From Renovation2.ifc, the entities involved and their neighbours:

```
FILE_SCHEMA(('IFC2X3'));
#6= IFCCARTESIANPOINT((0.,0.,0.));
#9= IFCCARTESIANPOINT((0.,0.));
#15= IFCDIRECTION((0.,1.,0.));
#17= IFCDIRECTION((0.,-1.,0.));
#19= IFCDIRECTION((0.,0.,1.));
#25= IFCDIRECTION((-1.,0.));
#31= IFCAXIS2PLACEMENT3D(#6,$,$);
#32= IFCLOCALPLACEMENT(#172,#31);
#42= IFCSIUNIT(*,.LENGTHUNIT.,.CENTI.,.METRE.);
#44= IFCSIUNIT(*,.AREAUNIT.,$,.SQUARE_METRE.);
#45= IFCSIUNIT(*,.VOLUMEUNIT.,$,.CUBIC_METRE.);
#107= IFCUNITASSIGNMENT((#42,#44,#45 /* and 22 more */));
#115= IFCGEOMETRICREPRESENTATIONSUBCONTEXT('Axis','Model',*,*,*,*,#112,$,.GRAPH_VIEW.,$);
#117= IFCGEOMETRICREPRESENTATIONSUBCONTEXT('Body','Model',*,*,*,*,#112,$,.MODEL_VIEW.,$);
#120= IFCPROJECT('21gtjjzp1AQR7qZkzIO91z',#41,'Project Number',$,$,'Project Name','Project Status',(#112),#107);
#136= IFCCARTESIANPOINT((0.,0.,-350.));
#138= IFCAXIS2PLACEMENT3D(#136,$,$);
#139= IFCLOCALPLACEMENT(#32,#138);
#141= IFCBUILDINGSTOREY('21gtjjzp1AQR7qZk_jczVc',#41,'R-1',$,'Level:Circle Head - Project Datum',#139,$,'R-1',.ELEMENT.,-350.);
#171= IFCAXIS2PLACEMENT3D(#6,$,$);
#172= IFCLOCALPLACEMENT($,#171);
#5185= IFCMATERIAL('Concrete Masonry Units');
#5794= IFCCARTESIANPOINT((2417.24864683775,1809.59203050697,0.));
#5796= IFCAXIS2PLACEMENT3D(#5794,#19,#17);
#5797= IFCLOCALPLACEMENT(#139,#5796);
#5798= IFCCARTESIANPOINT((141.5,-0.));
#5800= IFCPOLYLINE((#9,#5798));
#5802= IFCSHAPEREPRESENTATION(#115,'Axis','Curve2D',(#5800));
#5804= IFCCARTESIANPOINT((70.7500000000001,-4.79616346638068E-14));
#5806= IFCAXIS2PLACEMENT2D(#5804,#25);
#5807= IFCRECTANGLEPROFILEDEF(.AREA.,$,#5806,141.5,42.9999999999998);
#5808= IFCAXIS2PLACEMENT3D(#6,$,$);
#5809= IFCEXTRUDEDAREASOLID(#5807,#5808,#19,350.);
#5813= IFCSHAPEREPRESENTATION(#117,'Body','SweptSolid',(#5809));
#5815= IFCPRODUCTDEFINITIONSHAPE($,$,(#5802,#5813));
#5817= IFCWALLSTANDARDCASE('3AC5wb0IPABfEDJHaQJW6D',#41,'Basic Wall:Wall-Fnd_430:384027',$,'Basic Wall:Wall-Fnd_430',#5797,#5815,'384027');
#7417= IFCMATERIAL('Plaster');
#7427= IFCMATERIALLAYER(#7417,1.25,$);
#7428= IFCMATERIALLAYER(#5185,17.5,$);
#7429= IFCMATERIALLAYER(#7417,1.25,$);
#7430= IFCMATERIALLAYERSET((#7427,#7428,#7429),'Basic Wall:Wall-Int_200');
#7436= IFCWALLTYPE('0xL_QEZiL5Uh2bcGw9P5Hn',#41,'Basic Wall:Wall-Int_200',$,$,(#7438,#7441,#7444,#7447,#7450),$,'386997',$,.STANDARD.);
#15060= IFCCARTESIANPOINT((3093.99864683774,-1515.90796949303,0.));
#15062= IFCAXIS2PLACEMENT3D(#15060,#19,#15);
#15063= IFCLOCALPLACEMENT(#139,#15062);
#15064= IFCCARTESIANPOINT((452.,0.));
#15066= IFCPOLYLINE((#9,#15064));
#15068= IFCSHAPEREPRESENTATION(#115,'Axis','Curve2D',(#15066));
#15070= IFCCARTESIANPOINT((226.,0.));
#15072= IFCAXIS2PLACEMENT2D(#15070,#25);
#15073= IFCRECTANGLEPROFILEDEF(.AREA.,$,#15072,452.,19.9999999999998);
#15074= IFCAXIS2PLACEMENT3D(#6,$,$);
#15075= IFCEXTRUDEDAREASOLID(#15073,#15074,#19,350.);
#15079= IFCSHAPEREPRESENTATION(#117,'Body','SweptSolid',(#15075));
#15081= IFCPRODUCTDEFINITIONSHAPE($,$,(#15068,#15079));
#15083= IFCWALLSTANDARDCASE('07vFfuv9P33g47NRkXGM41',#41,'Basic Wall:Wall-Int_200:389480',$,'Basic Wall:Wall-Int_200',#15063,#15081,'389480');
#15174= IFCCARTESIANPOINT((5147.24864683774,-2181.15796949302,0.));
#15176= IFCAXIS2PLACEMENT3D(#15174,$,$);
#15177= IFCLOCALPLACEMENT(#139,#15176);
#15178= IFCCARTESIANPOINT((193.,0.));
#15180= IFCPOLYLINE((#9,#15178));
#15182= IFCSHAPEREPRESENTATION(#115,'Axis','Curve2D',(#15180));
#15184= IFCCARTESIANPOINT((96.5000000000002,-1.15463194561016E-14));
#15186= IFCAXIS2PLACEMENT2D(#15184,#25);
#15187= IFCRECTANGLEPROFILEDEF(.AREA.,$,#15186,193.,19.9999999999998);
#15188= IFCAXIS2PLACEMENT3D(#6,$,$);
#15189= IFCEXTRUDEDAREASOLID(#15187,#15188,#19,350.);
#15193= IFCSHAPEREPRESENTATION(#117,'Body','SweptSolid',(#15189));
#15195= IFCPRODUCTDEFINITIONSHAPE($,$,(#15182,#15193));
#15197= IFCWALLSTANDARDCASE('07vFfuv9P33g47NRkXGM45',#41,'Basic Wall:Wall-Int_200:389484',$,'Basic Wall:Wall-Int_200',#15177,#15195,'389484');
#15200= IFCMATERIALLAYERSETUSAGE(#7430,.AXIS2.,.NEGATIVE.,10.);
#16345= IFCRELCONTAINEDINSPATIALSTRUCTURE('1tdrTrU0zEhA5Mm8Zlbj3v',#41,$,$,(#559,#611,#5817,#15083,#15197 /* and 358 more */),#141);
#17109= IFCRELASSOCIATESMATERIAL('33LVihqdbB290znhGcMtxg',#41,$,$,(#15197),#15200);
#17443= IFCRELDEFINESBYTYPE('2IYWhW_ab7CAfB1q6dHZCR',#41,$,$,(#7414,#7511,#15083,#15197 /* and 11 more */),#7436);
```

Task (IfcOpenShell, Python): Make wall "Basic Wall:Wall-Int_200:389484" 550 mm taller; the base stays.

```python
import ifcopenshell
import ifcopenshell.geom
import ifcopenshell.util.representation
import ifcopenshell.util.shape
import ifcopenshell.util.unit

model = ifcopenshell.open("Renovation2.ifc")
unit_scale = ifcopenshell.util.unit.calculate_unit_scale(model)
settings = ifcopenshell.geom.settings()


def volume(element):
    """Net volume in cubic metres, openings subtracted."""
    shape = ifcopenshell.geom.create_shape(settings, element)
    return ifcopenshell.util.shape.get_volume(shape.geometry)


wall = model.by_guid("07vFfuv9P33g47NRkXGM45")
before = volume(wall)

body = ifcopenshell.util.representation.get_representation(wall, "Model", "Body")
solid = body.Items[0]
old_height = solid.Depth
solid.Depth += 0.55 / unit_scale
after = volume(wall)

print(f"height {old_height:g} -> {solid.Depth:g}, volume {before:.3f} -> {after:.3f} m3")

model.write("Renovation2_v2.ifc")
```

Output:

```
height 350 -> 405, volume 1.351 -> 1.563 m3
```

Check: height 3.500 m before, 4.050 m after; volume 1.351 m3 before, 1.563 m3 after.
